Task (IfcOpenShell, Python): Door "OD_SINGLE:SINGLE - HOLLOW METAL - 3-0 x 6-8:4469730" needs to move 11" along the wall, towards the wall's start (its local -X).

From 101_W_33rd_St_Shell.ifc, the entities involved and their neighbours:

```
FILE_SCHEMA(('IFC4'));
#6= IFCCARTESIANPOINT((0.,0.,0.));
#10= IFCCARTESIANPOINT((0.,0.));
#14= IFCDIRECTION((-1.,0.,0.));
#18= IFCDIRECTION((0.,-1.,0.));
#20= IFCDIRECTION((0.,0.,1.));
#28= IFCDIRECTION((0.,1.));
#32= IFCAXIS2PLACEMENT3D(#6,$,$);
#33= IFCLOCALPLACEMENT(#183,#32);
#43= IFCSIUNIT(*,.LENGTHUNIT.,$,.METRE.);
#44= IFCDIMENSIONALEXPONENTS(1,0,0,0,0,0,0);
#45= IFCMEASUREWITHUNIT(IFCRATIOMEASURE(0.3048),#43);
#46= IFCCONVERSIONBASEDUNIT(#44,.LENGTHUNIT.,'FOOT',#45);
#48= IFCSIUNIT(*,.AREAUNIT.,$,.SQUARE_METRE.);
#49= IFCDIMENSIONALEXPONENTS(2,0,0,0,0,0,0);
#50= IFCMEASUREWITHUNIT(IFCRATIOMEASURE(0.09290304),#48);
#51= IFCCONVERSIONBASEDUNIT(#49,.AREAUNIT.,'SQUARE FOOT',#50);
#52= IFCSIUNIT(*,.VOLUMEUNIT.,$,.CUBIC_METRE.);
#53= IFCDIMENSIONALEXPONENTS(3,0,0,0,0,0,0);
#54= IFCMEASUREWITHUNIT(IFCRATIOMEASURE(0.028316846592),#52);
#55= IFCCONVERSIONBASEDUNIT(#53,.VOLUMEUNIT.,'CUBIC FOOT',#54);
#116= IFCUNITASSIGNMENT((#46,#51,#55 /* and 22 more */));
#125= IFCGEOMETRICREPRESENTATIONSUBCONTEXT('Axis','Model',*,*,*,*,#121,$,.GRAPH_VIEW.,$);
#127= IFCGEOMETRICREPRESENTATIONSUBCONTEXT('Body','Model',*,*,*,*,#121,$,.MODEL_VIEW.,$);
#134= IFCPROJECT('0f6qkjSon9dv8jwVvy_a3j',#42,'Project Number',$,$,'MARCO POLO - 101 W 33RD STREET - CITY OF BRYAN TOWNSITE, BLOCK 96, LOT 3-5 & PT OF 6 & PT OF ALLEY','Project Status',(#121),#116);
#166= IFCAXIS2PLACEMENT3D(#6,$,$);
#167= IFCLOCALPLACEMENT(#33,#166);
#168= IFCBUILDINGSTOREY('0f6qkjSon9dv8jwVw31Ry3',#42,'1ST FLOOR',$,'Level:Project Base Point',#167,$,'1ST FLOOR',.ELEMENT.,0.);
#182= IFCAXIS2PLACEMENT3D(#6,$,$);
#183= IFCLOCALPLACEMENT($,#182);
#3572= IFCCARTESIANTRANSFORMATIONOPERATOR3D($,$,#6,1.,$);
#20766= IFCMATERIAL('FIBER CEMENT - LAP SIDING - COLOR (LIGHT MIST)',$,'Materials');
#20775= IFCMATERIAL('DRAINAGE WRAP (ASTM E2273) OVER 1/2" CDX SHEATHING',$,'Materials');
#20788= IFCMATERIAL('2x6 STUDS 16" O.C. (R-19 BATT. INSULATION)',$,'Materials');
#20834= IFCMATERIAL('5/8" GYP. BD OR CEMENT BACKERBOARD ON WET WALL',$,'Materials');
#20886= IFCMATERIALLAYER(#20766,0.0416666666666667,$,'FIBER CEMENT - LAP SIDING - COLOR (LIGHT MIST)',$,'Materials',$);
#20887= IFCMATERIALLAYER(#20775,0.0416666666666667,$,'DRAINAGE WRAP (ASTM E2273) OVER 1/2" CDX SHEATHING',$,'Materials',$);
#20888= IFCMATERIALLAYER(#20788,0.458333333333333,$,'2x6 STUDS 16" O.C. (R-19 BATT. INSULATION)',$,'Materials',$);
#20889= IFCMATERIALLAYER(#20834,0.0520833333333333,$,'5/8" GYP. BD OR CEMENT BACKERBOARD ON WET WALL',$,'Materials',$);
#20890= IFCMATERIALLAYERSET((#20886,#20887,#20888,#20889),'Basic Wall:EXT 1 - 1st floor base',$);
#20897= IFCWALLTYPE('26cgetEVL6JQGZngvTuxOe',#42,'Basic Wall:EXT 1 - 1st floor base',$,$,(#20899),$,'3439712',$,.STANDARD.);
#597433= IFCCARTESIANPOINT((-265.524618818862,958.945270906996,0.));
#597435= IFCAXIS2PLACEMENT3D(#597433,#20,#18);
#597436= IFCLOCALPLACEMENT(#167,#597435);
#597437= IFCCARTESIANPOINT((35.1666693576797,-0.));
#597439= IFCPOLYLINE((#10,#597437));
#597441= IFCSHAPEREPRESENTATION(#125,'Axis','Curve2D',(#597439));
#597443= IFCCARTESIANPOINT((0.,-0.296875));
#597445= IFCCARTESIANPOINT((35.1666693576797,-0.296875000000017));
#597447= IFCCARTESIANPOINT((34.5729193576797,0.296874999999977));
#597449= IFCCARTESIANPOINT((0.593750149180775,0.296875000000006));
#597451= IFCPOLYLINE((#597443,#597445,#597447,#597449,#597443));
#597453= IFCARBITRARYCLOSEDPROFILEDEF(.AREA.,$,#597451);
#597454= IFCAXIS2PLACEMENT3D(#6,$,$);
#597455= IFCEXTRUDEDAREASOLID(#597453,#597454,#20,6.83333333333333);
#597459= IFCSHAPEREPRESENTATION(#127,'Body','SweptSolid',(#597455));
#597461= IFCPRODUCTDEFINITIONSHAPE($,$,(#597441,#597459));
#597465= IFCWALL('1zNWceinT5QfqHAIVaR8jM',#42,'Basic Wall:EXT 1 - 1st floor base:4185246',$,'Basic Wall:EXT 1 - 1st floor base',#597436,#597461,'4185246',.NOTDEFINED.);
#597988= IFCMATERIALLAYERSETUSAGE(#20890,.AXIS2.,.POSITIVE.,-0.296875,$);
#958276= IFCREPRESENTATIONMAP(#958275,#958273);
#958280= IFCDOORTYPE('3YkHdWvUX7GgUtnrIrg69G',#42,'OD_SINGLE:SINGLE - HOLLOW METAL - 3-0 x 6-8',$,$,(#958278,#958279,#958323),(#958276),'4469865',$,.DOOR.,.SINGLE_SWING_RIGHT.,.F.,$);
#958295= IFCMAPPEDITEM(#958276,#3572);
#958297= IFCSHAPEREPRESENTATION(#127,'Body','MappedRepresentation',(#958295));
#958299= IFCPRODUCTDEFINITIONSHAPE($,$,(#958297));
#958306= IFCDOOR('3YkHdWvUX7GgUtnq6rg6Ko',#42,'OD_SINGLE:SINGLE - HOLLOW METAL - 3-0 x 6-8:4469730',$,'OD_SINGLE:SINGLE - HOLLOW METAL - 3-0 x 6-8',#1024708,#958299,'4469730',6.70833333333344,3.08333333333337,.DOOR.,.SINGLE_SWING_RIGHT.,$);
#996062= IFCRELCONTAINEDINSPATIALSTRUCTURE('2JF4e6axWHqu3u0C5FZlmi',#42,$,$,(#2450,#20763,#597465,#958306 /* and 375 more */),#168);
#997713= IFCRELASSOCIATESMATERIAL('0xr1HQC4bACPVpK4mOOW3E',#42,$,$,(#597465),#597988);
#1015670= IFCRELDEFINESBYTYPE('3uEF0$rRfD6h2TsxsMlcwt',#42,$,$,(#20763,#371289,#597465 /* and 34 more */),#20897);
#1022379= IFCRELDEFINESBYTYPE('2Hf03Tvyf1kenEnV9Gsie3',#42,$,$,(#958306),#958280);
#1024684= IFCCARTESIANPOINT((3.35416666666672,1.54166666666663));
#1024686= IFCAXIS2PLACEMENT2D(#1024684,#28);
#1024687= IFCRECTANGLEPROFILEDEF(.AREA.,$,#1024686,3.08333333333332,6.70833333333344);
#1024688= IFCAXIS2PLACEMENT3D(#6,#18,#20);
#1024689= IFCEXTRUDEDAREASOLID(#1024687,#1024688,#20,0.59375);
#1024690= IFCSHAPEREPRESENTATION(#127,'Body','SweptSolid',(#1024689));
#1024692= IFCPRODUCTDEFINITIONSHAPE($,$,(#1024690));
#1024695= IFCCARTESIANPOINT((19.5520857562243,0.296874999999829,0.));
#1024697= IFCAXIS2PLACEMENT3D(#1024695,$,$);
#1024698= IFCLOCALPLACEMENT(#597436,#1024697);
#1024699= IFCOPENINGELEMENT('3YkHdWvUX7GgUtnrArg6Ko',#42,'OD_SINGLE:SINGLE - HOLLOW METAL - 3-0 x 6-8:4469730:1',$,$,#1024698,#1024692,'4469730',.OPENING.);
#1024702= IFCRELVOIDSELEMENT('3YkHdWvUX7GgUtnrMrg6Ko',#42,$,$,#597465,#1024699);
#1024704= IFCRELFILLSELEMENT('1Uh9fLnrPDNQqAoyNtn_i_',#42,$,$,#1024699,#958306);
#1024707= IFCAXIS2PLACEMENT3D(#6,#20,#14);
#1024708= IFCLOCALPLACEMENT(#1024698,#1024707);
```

```python
import ifcopenshell
import ifcopenshell.api.geometry
import ifcopenshell.util.placement
import ifcopenshell.util.unit

model = ifcopenshell.open("101_W_33rd_St_Shell.ifc")
unit_scale = ifcopenshell.util.unit.calculate_unit_scale(model)

door = model.by_id(958306)
opening = door.FillsVoids[0].RelatingOpeningElement
wall = opening.VoidsElements[0].RelatingBuildingElement

wall_matrix = ifcopenshell.util.placement.get_local_placement(wall.ObjectPlacement)
shift = wall_matrix[:3, 0] * -11 * 0.0254 / unit_scale
before = ifcopenshell.util.placement.get_local_placement(door.ObjectPlacement)[:3, 3].copy()

# The door is placed relative to its opening, so it follows when the opening moves.
matrix = ifcopenshell.util.placement.get_local_placement(opening.ObjectPlacement)
matrix[:3, 3] += shift
ifcopenshell.api.geometry.edit_object_placement(
    model, product=opening, matrix=matrix, is_si=False, should_transform_children=True
)

after = ifcopenshell.util.placement.get_local_placement(door.ObjectPlacement)[:3, 3]
print("door moved by", (after - before).round(3) + 0.0)

model.write("101_W_33rd_St_Shell-out.ifc")
```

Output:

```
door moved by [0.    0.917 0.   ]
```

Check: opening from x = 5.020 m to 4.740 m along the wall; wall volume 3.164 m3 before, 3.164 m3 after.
